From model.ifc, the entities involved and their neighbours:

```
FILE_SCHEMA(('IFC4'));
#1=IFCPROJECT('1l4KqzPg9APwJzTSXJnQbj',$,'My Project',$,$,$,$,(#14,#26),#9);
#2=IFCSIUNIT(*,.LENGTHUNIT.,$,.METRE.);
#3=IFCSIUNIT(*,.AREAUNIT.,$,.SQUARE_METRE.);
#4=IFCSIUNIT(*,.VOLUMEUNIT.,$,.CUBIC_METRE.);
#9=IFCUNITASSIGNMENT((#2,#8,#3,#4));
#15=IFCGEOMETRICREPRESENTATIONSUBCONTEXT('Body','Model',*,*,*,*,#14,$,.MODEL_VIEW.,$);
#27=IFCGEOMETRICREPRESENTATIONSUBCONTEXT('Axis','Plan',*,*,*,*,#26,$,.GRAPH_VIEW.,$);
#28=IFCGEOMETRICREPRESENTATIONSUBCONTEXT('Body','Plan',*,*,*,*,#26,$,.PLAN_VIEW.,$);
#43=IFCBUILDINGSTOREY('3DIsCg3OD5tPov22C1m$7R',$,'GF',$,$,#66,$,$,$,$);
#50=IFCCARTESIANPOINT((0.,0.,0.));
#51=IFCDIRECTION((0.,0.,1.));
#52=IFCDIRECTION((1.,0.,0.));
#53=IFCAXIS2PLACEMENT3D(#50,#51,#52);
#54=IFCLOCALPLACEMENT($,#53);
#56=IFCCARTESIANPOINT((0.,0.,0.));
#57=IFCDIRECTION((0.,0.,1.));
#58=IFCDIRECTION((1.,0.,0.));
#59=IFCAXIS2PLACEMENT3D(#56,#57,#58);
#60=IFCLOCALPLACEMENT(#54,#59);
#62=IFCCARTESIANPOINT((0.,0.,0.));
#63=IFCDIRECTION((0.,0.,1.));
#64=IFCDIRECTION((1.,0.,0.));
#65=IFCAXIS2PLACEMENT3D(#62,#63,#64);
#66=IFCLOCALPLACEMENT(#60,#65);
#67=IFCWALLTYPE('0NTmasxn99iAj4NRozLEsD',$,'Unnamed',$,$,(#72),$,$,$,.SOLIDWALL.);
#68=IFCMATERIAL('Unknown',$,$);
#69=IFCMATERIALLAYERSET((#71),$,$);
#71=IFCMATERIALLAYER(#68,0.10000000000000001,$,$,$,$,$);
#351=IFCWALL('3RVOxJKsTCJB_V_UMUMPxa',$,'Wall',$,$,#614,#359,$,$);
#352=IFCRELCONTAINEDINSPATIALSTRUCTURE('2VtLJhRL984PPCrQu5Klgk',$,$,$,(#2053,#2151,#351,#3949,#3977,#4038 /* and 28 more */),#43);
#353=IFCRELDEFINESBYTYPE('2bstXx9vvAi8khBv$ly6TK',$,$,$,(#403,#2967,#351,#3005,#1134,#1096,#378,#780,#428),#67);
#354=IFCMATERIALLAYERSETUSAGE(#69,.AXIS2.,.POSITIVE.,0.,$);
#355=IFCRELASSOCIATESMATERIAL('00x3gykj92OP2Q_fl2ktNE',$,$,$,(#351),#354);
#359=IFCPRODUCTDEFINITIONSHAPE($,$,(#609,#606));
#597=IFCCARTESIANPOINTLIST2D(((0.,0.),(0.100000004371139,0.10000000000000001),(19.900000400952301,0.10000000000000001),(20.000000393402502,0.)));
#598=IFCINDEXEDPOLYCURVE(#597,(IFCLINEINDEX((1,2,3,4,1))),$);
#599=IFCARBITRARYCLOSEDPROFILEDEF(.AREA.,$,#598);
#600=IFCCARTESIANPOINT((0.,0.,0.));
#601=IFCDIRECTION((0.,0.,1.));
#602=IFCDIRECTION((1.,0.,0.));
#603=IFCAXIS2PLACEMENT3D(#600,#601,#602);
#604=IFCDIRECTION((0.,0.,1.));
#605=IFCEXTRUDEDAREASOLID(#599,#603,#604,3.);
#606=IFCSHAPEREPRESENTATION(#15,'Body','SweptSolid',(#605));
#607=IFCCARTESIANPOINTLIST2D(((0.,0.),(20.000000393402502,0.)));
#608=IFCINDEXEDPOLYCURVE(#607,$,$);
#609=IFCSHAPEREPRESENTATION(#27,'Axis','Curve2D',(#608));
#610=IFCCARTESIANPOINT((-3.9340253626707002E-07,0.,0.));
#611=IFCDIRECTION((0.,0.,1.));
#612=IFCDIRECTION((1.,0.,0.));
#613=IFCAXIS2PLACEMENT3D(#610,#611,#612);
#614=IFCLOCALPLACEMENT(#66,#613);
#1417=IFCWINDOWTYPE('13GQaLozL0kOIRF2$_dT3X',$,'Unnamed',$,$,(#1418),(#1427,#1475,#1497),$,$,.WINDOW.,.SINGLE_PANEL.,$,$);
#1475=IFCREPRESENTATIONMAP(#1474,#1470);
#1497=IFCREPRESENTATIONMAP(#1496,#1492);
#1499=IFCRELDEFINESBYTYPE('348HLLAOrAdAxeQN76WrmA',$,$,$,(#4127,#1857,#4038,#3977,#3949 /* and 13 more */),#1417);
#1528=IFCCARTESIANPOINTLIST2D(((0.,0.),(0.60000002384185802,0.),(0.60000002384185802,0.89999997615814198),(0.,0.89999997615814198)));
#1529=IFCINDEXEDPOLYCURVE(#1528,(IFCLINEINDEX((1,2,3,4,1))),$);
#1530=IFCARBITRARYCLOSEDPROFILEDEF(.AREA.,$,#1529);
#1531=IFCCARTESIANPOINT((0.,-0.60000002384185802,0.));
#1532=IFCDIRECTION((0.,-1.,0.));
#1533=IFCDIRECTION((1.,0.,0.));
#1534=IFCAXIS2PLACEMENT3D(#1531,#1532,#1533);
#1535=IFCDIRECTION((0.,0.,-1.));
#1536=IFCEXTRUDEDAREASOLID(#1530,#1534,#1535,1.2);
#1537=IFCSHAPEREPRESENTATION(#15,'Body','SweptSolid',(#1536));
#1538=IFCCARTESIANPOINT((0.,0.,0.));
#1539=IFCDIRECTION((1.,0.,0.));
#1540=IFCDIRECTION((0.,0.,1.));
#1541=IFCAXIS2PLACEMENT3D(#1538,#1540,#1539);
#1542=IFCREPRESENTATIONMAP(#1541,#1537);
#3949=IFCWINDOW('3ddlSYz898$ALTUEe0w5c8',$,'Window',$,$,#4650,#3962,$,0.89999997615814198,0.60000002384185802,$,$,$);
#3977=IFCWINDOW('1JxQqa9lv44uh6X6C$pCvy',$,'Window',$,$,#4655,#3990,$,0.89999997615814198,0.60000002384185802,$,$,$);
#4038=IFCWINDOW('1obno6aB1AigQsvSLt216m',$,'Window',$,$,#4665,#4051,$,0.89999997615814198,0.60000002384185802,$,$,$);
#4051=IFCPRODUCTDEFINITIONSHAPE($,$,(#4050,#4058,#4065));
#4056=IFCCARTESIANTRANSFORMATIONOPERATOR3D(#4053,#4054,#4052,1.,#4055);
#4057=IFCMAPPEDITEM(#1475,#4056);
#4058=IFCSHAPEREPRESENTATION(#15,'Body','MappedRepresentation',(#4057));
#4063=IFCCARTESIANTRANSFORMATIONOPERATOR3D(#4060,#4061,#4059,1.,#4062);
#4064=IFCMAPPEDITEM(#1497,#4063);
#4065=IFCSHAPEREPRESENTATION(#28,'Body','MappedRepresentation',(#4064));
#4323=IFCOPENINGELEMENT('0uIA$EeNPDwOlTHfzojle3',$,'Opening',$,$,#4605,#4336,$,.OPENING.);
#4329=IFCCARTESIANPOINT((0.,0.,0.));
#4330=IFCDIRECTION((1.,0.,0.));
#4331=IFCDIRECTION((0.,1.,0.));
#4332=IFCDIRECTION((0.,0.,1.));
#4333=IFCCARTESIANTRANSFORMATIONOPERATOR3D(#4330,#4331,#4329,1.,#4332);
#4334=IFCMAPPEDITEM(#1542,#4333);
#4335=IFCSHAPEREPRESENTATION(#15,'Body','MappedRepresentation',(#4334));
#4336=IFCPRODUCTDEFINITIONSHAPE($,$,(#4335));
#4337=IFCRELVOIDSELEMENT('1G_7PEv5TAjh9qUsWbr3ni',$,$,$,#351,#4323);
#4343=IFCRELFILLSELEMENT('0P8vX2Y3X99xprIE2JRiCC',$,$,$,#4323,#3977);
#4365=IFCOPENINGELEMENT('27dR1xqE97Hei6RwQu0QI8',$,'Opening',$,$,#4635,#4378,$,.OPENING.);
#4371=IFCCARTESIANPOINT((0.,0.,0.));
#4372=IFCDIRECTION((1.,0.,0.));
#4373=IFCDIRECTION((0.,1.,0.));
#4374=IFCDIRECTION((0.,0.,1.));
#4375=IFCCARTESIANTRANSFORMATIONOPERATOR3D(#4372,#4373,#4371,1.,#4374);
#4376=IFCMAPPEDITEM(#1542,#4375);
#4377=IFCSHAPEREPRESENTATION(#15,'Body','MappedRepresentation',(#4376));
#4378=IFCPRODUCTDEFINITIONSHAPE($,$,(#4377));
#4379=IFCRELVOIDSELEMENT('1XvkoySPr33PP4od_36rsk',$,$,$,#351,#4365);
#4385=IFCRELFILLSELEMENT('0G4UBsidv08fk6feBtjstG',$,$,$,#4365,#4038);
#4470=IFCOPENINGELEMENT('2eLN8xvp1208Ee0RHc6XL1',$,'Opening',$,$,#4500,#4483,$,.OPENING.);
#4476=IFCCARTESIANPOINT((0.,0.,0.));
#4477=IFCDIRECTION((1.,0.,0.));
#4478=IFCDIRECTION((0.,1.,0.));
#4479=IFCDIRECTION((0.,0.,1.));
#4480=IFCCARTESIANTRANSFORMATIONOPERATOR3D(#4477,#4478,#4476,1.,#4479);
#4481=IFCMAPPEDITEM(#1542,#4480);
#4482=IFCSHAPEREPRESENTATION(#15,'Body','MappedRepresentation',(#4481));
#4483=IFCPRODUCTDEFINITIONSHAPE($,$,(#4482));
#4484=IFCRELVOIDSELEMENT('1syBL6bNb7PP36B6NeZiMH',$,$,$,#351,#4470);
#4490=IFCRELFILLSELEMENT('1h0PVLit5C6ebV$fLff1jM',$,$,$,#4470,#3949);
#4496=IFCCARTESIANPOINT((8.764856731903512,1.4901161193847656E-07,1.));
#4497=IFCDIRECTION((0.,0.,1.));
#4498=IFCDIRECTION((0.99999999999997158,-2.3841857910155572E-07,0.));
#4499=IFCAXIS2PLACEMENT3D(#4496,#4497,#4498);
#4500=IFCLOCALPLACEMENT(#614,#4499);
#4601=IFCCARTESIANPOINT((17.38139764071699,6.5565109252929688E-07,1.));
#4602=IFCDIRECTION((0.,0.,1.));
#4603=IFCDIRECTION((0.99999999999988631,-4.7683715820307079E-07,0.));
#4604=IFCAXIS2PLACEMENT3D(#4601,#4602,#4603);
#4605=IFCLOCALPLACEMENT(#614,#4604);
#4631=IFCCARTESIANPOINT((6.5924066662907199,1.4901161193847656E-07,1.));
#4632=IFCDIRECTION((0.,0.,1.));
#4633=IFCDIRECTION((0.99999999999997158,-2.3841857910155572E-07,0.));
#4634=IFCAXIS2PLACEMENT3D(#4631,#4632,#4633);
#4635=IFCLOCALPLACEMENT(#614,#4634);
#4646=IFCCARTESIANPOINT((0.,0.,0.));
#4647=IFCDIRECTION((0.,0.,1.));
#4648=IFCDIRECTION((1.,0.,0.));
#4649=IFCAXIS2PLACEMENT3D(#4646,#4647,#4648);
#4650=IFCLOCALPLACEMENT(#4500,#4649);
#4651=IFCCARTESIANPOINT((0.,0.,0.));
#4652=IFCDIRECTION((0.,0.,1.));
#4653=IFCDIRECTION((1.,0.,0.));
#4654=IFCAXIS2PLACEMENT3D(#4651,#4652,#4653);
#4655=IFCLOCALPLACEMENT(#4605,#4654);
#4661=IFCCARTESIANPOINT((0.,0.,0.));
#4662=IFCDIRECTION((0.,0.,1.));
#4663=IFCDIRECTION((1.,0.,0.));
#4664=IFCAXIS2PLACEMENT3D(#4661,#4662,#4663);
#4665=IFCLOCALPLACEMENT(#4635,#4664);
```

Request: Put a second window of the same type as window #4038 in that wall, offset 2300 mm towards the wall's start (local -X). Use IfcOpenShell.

```python
import ifcopenshell
import ifcopenshell.api.feature
import ifcopenshell.api.geometry
import ifcopenshell.api.root
import ifcopenshell.geom
import ifcopenshell.util.element
import ifcopenshell.util.placement
import ifcopenshell.util.shape

model = ifcopenshell.open("model.ifc")
settings = ifcopenshell.geom.settings()


def volume(element):
    """Net volume in cubic metres, openings subtracted."""
    shape = ifcopenshell.geom.create_shape(settings, element)
    return ifcopenshell.util.shape.get_volume(shape.geometry)


window = model.by_guid("1obno6aB1AigQsvSLt216m")
opening = window.FillsVoids[0].RelatingOpeningElement
wall = opening.VoidsElements[0].RelatingBuildingElement
before = volume(wall)
shift = ifcopenshell.util.placement.get_local_placement(wall.ObjectPlacement)[:3, 0] * -2.3

# copy_class copies the void relationship, type, container and properties, but no geometry.
new_opening = ifcopenshell.api.root.copy_class(model, product=opening)
new_opening.Representation = ifcopenshell.util.element.copy_deep(
    model, opening.Representation, exclude=["IfcGeometricRepresentationContext", "IfcRepresentationMap"]
)
new_window = ifcopenshell.api.root.copy_class(model, product=window)
new_window.Representation = ifcopenshell.util.element.copy_deep(
    model, window.Representation, exclude=["IfcGeometricRepresentationContext", "IfcRepresentationMap"]
)
ifcopenshell.api.feature.add_filling(model, opening=new_opening, element=new_window)

for old, new in ((opening, new_opening), (window, new_window)):
    matrix = ifcopenshell.util.placement.get_local_placement(old.ObjectPlacement)
    matrix[:3, 3] += shift
    ifcopenshell.api.geometry.edit_object_placement(model, product=new, matrix=matrix, is_si=False)

after = volume(wall)

print(f"wall volume {before:.3f} -> {after:.3f} m3")

model.write("model_rev.ifc")
```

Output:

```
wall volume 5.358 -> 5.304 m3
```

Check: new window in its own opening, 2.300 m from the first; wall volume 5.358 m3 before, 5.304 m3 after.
